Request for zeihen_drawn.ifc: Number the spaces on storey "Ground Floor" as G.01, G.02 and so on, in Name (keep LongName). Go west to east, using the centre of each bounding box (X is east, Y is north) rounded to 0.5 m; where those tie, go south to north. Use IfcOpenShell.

First a look at what the model holds.

```python
import ifcopenshell
import ifcopenshell.util.element
import ifcopenshell.util.placement

model = ifcopenshell.open("zeihen_drawn.ifc")
print(model.schema)
storey = next(s for s in model.by_type("IfcBuildingStorey") if s.Name == "Ground Floor")
spaces = [e for e in ifcopenshell.util.element.get_decomposition(storey) if e.is_a("IfcSpace")]
for e in sorted(spaces, key=lambda e: e.id()):
    origin = ifcopenshell.util.placement.get_local_placement(e.ObjectPlacement)[:3, 3]
    print(e.id(), e.Name, e.LongName, origin.round(2) + 0.0, sep=" | ")
```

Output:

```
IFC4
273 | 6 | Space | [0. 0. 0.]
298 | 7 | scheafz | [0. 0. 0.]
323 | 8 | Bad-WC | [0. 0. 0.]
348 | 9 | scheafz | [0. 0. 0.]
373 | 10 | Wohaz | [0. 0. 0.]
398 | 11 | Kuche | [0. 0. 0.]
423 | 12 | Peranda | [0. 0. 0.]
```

```python
import ifcopenshell
import ifcopenshell.geom
import ifcopenshell.util.element
import ifcopenshell.util.shape

model = ifcopenshell.open("zeihen_drawn.ifc")
settings = ifcopenshell.geom.settings()
settings.set("use-world-coords", True)


def centre(element):
    shape = ifcopenshell.geom.create_shape(settings, element)
    return ifcopenshell.util.shape.get_bbox_centroid(shape.geometry)


storey = next(s for s in model.by_type("IfcBuildingStorey") if s.Name == "Ground Floor")
spaces = [e for e in ifcopenshell.util.element.get_decomposition(storey) if e.is_a("IfcSpace")]

# Insertion points can sit at a corner or the storey origin, so sort by the geometry (in metres).
centres = {e: centre(e) for e in spaces}
spaces.sort(key=lambda e: (round(centres[e][0] / 0.5), centres[e][1]))

for i, e in enumerate(spaces, start=1):
    number = f"G.{i:02d}"
    e.Name = number
    print(e.id(), number)

model.write("zeihen_drawn_edited.ifc")
```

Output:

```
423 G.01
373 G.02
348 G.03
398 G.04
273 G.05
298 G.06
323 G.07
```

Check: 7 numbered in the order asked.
